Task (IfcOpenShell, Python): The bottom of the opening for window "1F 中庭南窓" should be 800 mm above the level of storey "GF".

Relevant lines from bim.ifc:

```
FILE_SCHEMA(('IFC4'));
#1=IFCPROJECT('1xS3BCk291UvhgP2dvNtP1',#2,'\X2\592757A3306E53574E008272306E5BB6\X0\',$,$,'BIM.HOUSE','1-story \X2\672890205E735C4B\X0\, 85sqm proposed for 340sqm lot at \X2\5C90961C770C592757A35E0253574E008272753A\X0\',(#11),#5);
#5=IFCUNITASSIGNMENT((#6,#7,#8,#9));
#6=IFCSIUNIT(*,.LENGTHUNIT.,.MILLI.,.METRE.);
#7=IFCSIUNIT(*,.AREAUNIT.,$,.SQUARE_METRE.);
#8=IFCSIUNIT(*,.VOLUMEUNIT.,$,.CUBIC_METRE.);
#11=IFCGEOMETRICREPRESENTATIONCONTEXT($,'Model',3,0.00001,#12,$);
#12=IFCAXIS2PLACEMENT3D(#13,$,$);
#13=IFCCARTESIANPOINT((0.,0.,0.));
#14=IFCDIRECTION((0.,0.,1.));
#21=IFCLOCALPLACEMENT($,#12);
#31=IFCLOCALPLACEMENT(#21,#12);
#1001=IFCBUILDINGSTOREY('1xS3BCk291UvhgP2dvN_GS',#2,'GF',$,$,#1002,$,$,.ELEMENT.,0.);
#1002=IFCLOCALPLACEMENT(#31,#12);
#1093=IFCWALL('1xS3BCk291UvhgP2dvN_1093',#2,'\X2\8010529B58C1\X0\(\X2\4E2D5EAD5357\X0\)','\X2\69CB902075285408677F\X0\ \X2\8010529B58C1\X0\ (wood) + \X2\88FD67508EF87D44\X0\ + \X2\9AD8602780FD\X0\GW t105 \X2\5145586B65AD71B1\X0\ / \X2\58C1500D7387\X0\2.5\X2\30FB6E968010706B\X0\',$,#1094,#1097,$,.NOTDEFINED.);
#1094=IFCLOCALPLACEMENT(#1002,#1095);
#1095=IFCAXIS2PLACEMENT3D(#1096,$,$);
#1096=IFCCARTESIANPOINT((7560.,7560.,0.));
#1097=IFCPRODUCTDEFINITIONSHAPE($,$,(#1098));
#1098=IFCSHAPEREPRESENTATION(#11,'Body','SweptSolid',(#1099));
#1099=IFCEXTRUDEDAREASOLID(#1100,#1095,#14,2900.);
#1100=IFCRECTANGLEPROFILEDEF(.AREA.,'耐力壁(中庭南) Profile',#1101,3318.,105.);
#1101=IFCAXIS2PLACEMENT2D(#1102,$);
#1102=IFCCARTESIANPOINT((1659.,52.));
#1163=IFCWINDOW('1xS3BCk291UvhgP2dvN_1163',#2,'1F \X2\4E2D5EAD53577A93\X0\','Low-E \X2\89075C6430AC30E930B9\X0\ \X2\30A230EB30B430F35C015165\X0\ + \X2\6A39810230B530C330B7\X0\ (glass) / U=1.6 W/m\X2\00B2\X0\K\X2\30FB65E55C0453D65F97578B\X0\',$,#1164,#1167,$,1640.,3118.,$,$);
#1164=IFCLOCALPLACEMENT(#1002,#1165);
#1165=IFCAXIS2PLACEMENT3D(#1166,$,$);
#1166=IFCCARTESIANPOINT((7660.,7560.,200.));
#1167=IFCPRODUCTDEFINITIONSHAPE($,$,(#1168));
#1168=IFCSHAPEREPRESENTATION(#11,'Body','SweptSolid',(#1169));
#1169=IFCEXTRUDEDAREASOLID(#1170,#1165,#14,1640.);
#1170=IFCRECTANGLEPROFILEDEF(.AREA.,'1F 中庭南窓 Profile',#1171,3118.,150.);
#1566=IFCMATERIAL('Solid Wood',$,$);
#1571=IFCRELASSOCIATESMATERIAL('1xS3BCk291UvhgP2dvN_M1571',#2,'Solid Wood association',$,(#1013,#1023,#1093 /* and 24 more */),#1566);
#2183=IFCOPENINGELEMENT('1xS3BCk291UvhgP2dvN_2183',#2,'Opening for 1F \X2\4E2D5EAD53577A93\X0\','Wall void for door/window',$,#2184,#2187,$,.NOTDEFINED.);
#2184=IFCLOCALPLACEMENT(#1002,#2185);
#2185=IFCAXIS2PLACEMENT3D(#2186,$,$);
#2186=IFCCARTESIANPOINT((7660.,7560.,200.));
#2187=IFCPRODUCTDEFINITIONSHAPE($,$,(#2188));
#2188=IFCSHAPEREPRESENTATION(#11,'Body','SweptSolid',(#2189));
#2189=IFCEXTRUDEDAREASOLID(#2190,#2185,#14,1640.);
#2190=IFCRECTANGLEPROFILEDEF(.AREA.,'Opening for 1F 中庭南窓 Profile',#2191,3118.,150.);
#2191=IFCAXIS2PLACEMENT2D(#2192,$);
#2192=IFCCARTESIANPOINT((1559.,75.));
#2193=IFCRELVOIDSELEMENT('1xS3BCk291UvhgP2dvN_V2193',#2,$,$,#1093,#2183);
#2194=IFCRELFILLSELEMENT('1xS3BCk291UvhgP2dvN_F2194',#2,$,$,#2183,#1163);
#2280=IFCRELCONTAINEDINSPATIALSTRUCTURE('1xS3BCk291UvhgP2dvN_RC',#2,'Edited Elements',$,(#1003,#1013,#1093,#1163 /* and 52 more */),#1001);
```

```python
import numpy as np
import ifcopenshell
import ifcopenshell.api.geometry
import ifcopenshell.geom
import ifcopenshell.util.element
import ifcopenshell.util.placement
import ifcopenshell.util.shape
import ifcopenshell.util.unit

model = ifcopenshell.open("bim.ifc")
unit_scale = ifcopenshell.util.unit.calculate_unit_scale(model)

window = model.by_id(1163)
opening = window.FillsVoids[0].RelatingOpeningElement
storey = ifcopenshell.util.element.get_container(window, ifc_class="IfcBuildingStorey")
level = ifcopenshell.util.placement.get_local_placement(storey.ObjectPlacement)[2, 3]

# The opening's origin need not be at the sill, so measure its lowest point.
shape = ifcopenshell.geom.create_shape(ifcopenshell.geom.settings(), opening)
bottom = ifcopenshell.util.shape.get_shape_bottom_elevation(shape, shape.geometry) / unit_scale
dz = level + 0.8 / unit_scale - bottom

shift = np.array([0.0, 0.0, dz])
# The window is not placed relative to its opening, so move both.
for product in (opening, window):
    matrix = ifcopenshell.util.placement.get_local_placement(product.ObjectPlacement)
    matrix[:3, 3] += shift
    ifcopenshell.api.geometry.edit_object_placement(model, product=product, matrix=matrix, is_si=False)

print(f"moved by {dz * unit_scale:+.3f} m")

model.write("bim_updated.ifc")
```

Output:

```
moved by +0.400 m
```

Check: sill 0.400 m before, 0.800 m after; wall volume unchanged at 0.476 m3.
